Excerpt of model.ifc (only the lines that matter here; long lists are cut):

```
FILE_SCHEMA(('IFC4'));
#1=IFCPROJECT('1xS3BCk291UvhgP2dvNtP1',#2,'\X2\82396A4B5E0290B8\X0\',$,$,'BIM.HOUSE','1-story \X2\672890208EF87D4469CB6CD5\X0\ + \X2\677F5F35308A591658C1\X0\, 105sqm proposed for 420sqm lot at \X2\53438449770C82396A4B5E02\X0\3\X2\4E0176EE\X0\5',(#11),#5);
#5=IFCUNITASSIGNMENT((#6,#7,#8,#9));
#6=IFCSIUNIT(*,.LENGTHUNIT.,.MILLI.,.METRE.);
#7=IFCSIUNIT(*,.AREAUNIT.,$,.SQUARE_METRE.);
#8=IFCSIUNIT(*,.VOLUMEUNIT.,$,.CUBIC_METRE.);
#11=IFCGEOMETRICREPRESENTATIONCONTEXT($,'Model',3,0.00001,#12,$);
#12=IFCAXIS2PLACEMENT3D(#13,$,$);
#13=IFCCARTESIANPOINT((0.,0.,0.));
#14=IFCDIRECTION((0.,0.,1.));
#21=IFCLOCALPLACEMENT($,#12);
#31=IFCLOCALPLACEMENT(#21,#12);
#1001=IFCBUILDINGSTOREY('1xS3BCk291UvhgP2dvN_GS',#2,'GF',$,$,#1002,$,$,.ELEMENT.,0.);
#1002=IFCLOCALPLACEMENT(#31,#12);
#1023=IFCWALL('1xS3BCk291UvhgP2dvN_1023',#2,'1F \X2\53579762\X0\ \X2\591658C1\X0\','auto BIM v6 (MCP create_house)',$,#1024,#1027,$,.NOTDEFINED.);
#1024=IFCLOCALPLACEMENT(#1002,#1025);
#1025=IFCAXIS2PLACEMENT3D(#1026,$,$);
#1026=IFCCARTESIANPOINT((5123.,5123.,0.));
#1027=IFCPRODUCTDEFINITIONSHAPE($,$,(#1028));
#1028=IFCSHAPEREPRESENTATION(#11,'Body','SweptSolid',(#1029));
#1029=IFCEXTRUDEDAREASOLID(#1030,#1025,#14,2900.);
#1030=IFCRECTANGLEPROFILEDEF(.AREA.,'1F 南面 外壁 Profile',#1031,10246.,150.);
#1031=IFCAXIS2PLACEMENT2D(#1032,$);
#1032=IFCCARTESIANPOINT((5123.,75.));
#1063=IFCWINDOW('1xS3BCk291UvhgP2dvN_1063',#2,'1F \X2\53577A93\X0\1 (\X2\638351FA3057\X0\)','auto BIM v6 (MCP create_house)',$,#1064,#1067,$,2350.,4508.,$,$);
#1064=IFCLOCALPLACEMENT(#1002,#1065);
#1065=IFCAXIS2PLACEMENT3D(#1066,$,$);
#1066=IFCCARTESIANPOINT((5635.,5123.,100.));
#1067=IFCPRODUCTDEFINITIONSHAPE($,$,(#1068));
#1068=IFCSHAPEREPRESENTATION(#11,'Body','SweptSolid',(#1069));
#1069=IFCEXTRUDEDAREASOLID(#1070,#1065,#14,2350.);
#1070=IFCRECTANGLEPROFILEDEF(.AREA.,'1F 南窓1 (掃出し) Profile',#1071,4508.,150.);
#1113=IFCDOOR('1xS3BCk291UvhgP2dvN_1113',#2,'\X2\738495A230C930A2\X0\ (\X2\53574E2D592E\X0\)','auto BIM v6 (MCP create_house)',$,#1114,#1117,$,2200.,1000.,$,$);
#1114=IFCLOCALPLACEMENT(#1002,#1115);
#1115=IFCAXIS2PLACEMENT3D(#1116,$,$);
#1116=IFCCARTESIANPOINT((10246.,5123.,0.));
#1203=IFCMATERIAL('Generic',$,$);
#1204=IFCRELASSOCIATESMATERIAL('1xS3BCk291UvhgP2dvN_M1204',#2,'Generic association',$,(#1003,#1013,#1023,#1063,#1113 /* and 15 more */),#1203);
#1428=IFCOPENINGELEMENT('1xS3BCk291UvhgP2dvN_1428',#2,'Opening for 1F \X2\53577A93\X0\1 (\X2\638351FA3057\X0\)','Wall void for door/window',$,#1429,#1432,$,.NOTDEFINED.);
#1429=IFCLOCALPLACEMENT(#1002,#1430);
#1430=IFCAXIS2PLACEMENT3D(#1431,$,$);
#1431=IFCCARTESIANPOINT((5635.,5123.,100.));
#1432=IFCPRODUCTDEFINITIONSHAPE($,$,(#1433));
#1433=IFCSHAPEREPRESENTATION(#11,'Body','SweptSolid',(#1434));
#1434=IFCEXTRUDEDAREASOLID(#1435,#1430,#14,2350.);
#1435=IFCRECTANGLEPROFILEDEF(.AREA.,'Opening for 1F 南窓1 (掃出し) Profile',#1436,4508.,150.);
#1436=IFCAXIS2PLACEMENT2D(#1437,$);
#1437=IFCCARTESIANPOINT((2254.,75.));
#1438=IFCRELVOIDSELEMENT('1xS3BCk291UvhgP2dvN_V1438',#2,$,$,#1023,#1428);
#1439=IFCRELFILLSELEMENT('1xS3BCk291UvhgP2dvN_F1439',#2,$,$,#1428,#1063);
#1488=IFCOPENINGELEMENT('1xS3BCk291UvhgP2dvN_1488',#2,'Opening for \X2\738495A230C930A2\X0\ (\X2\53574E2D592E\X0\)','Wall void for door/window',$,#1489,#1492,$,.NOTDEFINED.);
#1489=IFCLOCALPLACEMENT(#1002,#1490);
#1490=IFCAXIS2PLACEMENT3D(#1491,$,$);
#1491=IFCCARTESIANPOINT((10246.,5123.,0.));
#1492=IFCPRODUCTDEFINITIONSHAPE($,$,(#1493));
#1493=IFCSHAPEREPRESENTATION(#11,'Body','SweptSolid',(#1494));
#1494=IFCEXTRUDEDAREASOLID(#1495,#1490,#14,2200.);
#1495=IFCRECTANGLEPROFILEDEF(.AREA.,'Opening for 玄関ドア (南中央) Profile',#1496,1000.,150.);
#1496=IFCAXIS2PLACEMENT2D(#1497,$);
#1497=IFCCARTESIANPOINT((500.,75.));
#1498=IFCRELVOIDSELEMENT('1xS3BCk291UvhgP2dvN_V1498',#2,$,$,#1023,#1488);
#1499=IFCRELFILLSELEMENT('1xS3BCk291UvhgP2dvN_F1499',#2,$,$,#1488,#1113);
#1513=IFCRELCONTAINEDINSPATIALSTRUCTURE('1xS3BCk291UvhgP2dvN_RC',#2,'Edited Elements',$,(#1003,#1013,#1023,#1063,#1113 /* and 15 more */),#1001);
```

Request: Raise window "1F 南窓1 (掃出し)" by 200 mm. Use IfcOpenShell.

```python
import numpy as np
import ifcopenshell
import ifcopenshell.api.geometry
import ifcopenshell.util.placement
import ifcopenshell.util.unit

model = ifcopenshell.open("model.ifc")
unit_scale = ifcopenshell.util.unit.calculate_unit_scale(model)

window = model.by_id(1063)
opening = window.FillsVoids[0].RelatingOpeningElement
dz = 0.2 / unit_scale

shift = np.array([0.0, 0.0, dz])
# The window is not placed relative to its opening, so move both.
for product in (opening, window):
    matrix = ifcopenshell.util.placement.get_local_placement(product.ObjectPlacement)
    matrix[:3, 3] += shift
    ifcopenshell.api.geometry.edit_object_placement(model, product=product, matrix=matrix, is_si=False)

print(f"moved by {dz * unit_scale:+.3f} m")

model.write("model_updated.ifc")
```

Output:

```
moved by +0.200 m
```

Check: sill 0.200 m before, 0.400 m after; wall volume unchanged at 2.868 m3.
